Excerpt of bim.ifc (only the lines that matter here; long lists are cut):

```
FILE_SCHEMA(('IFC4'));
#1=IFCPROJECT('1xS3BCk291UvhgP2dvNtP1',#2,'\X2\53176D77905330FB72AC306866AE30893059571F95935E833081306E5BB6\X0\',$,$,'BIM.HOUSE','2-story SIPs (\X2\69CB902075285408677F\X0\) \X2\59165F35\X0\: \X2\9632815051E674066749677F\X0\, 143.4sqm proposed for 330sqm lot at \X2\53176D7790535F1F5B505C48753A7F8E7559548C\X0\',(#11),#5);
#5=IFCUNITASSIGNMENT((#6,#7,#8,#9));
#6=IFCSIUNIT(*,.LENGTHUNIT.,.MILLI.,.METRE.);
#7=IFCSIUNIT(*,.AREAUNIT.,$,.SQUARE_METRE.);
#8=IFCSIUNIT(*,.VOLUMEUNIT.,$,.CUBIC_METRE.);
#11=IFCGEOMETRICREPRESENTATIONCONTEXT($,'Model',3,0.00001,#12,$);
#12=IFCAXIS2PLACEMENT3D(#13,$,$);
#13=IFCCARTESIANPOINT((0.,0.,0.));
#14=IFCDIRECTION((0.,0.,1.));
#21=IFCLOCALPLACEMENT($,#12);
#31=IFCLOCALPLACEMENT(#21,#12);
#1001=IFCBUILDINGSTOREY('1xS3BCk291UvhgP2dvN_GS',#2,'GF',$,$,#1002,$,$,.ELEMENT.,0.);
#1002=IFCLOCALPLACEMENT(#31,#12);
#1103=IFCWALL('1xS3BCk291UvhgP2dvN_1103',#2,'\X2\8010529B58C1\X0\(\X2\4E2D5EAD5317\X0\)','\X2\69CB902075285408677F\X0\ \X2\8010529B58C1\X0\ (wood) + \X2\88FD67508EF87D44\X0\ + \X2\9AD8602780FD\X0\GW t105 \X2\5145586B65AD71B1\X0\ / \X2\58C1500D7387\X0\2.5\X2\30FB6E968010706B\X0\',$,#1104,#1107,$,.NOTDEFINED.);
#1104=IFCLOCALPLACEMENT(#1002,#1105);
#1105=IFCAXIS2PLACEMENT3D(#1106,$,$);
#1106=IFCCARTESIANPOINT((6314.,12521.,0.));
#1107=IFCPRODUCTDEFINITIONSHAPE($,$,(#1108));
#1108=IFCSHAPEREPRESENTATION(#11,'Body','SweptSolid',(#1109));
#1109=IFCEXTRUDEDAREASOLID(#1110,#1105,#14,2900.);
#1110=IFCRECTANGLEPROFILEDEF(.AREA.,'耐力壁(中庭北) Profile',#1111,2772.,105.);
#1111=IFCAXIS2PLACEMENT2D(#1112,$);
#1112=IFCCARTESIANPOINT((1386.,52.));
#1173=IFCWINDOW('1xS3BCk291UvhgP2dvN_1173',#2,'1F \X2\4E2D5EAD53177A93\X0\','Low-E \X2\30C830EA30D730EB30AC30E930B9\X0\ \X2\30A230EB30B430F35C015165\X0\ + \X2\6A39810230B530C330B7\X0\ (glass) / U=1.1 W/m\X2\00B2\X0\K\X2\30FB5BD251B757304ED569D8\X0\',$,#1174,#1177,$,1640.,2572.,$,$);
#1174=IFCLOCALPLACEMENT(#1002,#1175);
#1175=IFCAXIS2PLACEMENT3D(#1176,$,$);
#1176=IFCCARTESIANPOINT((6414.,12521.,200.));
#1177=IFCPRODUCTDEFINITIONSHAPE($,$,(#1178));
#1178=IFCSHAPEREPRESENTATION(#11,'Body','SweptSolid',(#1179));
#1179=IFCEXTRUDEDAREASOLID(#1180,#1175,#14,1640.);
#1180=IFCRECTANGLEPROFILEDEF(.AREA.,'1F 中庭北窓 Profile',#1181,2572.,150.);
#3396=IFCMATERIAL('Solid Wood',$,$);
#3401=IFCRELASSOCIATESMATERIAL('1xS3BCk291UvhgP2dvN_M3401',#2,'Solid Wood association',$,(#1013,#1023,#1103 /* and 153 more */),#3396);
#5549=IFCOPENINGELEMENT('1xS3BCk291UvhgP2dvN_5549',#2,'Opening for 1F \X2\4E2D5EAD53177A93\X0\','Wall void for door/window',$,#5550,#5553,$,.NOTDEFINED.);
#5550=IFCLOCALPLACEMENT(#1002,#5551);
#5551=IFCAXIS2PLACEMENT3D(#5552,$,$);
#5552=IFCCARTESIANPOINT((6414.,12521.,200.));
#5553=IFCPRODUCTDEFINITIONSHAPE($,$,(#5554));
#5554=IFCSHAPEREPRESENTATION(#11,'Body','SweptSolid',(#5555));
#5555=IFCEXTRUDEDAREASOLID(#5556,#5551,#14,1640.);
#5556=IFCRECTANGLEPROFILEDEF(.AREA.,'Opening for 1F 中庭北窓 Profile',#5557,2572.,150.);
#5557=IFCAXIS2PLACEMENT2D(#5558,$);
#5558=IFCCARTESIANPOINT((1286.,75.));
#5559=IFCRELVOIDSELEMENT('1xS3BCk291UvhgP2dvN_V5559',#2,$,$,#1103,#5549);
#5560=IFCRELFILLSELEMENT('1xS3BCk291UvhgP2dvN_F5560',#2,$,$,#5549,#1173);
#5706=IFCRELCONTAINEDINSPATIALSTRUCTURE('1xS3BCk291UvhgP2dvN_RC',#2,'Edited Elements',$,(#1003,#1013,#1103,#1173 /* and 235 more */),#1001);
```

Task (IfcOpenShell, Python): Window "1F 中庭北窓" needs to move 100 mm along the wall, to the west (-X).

```python
import ifcopenshell
import ifcopenshell.api.geometry
import ifcopenshell.util.placement
import ifcopenshell.util.unit

model = ifcopenshell.open("bim.ifc")
unit_scale = ifcopenshell.util.unit.calculate_unit_scale(model)

window = model.by_guid("1xS3BCk291UvhgP2dvN_1173")
opening = window.FillsVoids[0].RelatingOpeningElement
wall = opening.VoidsElements[0].RelatingBuildingElement

wall_matrix = ifcopenshell.util.placement.get_local_placement(wall.ObjectPlacement)
shift = wall_matrix[:3, 0] * -0.1 / unit_scale
before = ifcopenshell.util.placement.get_local_placement(window.ObjectPlacement)[:3, 3].copy()

# The window is not placed relative to its opening, so move both.
for product in (opening, window):
    matrix = ifcopenshell.util.placement.get_local_placement(product.ObjectPlacement)
    matrix[:3, 3] += shift
    ifcopenshell.api.geometry.edit_object_placement(model, product=product, matrix=matrix, is_si=False)

after = ifcopenshell.util.placement.get_local_placement(window.ObjectPlacement)[:3, 3]
print("window moved by", (after - before).round(3) + 0.0)

model.write("bim-out.ifc")
```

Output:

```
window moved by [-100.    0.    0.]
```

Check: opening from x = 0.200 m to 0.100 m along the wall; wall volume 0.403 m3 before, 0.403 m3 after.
